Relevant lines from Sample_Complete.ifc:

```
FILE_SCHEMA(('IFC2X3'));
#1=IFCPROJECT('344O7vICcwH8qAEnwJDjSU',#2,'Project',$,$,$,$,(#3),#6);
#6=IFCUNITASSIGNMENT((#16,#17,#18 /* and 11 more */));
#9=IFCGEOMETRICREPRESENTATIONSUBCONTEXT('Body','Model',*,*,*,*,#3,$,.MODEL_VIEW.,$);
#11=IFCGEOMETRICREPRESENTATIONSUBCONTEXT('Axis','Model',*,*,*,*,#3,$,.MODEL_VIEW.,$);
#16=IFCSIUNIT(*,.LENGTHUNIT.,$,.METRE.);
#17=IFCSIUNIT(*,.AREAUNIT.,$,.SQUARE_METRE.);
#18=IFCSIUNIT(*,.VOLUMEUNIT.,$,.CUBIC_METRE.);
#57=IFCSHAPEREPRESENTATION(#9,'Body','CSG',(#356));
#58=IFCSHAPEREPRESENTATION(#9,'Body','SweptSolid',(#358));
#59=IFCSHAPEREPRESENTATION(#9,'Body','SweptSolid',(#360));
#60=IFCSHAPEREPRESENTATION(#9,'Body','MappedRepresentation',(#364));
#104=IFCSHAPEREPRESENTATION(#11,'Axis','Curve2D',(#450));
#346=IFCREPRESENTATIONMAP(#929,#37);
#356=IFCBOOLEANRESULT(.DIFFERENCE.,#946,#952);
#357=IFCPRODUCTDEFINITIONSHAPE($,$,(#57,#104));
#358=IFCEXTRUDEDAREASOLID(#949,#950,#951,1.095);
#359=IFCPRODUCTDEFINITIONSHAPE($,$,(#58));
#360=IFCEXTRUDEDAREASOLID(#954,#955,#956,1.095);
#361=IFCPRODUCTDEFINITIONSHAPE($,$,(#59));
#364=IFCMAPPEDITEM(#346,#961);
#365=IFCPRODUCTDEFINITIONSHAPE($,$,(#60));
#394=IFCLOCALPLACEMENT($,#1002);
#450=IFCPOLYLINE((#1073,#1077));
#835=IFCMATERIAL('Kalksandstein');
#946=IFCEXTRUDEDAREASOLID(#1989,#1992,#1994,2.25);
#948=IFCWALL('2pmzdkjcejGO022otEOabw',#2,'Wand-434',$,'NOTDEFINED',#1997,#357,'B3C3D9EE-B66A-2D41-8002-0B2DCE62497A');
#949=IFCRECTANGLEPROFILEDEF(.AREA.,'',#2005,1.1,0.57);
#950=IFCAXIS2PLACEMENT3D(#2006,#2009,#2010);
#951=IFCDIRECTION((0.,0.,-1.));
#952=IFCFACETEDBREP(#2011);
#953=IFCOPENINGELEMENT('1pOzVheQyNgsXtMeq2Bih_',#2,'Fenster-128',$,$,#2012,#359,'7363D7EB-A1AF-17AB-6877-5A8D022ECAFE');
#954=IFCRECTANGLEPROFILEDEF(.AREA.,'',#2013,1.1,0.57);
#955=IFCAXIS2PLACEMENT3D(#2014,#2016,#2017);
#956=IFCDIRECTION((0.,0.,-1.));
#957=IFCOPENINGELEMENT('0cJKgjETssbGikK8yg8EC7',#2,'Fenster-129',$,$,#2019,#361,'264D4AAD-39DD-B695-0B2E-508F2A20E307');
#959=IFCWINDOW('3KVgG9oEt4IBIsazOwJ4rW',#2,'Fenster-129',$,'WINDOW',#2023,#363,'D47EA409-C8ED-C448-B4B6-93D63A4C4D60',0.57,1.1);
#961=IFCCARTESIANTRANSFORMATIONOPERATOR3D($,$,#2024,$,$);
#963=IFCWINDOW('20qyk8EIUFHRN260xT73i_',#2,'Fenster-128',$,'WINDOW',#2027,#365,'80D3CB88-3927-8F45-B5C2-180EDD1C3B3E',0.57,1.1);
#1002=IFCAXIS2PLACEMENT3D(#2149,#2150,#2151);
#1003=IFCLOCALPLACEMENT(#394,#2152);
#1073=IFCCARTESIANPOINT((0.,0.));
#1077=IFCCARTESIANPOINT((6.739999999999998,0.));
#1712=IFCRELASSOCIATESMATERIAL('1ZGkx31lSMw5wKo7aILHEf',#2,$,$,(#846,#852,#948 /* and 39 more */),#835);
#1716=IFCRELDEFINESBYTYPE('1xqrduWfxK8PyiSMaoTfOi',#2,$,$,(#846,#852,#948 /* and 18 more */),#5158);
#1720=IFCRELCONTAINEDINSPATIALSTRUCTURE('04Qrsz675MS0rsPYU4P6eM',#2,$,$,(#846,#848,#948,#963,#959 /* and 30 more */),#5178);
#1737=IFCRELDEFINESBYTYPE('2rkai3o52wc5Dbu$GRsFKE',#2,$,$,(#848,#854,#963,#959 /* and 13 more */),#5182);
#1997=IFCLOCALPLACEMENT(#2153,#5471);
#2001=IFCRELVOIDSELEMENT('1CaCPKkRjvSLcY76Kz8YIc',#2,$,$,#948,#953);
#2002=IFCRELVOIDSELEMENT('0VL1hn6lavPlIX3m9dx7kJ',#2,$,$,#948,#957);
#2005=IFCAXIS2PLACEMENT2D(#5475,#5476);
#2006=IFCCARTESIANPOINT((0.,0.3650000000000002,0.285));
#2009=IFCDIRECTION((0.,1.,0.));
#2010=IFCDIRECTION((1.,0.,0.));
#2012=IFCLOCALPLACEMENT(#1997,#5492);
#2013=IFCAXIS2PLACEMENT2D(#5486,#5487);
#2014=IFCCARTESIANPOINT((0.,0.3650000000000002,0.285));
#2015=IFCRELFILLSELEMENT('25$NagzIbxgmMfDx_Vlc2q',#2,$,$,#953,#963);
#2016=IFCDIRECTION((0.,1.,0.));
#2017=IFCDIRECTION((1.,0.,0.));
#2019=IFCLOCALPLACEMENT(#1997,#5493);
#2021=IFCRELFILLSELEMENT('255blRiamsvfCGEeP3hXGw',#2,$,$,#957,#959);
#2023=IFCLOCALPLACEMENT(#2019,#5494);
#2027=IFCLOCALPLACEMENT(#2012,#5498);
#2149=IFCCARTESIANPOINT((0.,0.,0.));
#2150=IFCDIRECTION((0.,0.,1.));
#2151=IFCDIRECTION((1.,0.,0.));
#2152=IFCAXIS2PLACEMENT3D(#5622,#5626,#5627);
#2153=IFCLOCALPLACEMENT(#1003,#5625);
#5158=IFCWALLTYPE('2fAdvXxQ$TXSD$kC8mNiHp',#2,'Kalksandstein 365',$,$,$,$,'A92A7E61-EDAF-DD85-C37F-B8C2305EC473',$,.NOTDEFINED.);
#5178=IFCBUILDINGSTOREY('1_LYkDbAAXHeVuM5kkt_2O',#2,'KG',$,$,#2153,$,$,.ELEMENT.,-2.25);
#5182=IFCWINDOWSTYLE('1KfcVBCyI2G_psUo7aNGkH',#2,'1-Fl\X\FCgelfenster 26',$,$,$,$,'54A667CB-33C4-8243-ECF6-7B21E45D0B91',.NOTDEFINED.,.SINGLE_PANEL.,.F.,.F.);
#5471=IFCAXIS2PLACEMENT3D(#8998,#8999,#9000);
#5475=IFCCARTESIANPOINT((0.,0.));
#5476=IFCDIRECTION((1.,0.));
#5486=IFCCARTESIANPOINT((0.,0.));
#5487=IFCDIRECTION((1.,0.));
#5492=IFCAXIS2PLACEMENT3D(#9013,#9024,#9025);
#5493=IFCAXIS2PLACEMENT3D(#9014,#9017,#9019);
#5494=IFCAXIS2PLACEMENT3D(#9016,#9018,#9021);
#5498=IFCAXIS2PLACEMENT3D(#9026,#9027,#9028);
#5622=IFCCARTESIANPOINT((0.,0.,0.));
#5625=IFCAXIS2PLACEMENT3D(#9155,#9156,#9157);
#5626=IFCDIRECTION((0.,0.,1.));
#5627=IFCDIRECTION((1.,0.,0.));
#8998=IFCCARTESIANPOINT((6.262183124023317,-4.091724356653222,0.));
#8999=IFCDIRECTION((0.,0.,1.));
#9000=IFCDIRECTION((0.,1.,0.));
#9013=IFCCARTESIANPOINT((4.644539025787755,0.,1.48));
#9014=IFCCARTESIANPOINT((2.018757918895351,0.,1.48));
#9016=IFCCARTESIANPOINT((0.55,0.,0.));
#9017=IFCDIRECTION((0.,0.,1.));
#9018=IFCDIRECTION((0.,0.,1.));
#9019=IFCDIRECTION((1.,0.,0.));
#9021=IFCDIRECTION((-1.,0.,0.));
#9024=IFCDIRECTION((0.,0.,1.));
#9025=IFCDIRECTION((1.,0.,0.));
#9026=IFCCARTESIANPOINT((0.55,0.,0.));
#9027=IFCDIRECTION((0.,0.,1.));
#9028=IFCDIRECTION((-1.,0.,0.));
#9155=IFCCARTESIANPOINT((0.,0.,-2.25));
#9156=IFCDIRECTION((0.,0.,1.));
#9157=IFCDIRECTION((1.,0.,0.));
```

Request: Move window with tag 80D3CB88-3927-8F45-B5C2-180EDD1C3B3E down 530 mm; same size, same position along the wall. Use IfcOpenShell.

```python
import numpy as np
import ifcopenshell
import ifcopenshell.api.geometry
import ifcopenshell.util.placement
import ifcopenshell.util.unit

model = ifcopenshell.open("Sample_Complete.ifc")
unit_scale = ifcopenshell.util.unit.calculate_unit_scale(model)

window = model.by_guid("20qyk8EIUFHRN260xT73i_")
opening = window.FillsVoids[0].RelatingOpeningElement
dz = -0.53

shift = np.array([0.0, 0.0, dz])
# The window is placed relative to its opening, so it follows when the opening moves.
matrix = ifcopenshell.util.placement.get_local_placement(opening.ObjectPlacement)
matrix[:3, 3] += shift
ifcopenshell.api.geometry.edit_object_placement(
    model, product=opening, matrix=matrix, is_si=False, should_transform_children=True
)

print(f"moved by {dz * unit_scale:+.3f} m")

model.write("Sample_Complete-out.ifc")
```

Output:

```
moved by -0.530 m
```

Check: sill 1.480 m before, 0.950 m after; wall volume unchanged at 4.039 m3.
